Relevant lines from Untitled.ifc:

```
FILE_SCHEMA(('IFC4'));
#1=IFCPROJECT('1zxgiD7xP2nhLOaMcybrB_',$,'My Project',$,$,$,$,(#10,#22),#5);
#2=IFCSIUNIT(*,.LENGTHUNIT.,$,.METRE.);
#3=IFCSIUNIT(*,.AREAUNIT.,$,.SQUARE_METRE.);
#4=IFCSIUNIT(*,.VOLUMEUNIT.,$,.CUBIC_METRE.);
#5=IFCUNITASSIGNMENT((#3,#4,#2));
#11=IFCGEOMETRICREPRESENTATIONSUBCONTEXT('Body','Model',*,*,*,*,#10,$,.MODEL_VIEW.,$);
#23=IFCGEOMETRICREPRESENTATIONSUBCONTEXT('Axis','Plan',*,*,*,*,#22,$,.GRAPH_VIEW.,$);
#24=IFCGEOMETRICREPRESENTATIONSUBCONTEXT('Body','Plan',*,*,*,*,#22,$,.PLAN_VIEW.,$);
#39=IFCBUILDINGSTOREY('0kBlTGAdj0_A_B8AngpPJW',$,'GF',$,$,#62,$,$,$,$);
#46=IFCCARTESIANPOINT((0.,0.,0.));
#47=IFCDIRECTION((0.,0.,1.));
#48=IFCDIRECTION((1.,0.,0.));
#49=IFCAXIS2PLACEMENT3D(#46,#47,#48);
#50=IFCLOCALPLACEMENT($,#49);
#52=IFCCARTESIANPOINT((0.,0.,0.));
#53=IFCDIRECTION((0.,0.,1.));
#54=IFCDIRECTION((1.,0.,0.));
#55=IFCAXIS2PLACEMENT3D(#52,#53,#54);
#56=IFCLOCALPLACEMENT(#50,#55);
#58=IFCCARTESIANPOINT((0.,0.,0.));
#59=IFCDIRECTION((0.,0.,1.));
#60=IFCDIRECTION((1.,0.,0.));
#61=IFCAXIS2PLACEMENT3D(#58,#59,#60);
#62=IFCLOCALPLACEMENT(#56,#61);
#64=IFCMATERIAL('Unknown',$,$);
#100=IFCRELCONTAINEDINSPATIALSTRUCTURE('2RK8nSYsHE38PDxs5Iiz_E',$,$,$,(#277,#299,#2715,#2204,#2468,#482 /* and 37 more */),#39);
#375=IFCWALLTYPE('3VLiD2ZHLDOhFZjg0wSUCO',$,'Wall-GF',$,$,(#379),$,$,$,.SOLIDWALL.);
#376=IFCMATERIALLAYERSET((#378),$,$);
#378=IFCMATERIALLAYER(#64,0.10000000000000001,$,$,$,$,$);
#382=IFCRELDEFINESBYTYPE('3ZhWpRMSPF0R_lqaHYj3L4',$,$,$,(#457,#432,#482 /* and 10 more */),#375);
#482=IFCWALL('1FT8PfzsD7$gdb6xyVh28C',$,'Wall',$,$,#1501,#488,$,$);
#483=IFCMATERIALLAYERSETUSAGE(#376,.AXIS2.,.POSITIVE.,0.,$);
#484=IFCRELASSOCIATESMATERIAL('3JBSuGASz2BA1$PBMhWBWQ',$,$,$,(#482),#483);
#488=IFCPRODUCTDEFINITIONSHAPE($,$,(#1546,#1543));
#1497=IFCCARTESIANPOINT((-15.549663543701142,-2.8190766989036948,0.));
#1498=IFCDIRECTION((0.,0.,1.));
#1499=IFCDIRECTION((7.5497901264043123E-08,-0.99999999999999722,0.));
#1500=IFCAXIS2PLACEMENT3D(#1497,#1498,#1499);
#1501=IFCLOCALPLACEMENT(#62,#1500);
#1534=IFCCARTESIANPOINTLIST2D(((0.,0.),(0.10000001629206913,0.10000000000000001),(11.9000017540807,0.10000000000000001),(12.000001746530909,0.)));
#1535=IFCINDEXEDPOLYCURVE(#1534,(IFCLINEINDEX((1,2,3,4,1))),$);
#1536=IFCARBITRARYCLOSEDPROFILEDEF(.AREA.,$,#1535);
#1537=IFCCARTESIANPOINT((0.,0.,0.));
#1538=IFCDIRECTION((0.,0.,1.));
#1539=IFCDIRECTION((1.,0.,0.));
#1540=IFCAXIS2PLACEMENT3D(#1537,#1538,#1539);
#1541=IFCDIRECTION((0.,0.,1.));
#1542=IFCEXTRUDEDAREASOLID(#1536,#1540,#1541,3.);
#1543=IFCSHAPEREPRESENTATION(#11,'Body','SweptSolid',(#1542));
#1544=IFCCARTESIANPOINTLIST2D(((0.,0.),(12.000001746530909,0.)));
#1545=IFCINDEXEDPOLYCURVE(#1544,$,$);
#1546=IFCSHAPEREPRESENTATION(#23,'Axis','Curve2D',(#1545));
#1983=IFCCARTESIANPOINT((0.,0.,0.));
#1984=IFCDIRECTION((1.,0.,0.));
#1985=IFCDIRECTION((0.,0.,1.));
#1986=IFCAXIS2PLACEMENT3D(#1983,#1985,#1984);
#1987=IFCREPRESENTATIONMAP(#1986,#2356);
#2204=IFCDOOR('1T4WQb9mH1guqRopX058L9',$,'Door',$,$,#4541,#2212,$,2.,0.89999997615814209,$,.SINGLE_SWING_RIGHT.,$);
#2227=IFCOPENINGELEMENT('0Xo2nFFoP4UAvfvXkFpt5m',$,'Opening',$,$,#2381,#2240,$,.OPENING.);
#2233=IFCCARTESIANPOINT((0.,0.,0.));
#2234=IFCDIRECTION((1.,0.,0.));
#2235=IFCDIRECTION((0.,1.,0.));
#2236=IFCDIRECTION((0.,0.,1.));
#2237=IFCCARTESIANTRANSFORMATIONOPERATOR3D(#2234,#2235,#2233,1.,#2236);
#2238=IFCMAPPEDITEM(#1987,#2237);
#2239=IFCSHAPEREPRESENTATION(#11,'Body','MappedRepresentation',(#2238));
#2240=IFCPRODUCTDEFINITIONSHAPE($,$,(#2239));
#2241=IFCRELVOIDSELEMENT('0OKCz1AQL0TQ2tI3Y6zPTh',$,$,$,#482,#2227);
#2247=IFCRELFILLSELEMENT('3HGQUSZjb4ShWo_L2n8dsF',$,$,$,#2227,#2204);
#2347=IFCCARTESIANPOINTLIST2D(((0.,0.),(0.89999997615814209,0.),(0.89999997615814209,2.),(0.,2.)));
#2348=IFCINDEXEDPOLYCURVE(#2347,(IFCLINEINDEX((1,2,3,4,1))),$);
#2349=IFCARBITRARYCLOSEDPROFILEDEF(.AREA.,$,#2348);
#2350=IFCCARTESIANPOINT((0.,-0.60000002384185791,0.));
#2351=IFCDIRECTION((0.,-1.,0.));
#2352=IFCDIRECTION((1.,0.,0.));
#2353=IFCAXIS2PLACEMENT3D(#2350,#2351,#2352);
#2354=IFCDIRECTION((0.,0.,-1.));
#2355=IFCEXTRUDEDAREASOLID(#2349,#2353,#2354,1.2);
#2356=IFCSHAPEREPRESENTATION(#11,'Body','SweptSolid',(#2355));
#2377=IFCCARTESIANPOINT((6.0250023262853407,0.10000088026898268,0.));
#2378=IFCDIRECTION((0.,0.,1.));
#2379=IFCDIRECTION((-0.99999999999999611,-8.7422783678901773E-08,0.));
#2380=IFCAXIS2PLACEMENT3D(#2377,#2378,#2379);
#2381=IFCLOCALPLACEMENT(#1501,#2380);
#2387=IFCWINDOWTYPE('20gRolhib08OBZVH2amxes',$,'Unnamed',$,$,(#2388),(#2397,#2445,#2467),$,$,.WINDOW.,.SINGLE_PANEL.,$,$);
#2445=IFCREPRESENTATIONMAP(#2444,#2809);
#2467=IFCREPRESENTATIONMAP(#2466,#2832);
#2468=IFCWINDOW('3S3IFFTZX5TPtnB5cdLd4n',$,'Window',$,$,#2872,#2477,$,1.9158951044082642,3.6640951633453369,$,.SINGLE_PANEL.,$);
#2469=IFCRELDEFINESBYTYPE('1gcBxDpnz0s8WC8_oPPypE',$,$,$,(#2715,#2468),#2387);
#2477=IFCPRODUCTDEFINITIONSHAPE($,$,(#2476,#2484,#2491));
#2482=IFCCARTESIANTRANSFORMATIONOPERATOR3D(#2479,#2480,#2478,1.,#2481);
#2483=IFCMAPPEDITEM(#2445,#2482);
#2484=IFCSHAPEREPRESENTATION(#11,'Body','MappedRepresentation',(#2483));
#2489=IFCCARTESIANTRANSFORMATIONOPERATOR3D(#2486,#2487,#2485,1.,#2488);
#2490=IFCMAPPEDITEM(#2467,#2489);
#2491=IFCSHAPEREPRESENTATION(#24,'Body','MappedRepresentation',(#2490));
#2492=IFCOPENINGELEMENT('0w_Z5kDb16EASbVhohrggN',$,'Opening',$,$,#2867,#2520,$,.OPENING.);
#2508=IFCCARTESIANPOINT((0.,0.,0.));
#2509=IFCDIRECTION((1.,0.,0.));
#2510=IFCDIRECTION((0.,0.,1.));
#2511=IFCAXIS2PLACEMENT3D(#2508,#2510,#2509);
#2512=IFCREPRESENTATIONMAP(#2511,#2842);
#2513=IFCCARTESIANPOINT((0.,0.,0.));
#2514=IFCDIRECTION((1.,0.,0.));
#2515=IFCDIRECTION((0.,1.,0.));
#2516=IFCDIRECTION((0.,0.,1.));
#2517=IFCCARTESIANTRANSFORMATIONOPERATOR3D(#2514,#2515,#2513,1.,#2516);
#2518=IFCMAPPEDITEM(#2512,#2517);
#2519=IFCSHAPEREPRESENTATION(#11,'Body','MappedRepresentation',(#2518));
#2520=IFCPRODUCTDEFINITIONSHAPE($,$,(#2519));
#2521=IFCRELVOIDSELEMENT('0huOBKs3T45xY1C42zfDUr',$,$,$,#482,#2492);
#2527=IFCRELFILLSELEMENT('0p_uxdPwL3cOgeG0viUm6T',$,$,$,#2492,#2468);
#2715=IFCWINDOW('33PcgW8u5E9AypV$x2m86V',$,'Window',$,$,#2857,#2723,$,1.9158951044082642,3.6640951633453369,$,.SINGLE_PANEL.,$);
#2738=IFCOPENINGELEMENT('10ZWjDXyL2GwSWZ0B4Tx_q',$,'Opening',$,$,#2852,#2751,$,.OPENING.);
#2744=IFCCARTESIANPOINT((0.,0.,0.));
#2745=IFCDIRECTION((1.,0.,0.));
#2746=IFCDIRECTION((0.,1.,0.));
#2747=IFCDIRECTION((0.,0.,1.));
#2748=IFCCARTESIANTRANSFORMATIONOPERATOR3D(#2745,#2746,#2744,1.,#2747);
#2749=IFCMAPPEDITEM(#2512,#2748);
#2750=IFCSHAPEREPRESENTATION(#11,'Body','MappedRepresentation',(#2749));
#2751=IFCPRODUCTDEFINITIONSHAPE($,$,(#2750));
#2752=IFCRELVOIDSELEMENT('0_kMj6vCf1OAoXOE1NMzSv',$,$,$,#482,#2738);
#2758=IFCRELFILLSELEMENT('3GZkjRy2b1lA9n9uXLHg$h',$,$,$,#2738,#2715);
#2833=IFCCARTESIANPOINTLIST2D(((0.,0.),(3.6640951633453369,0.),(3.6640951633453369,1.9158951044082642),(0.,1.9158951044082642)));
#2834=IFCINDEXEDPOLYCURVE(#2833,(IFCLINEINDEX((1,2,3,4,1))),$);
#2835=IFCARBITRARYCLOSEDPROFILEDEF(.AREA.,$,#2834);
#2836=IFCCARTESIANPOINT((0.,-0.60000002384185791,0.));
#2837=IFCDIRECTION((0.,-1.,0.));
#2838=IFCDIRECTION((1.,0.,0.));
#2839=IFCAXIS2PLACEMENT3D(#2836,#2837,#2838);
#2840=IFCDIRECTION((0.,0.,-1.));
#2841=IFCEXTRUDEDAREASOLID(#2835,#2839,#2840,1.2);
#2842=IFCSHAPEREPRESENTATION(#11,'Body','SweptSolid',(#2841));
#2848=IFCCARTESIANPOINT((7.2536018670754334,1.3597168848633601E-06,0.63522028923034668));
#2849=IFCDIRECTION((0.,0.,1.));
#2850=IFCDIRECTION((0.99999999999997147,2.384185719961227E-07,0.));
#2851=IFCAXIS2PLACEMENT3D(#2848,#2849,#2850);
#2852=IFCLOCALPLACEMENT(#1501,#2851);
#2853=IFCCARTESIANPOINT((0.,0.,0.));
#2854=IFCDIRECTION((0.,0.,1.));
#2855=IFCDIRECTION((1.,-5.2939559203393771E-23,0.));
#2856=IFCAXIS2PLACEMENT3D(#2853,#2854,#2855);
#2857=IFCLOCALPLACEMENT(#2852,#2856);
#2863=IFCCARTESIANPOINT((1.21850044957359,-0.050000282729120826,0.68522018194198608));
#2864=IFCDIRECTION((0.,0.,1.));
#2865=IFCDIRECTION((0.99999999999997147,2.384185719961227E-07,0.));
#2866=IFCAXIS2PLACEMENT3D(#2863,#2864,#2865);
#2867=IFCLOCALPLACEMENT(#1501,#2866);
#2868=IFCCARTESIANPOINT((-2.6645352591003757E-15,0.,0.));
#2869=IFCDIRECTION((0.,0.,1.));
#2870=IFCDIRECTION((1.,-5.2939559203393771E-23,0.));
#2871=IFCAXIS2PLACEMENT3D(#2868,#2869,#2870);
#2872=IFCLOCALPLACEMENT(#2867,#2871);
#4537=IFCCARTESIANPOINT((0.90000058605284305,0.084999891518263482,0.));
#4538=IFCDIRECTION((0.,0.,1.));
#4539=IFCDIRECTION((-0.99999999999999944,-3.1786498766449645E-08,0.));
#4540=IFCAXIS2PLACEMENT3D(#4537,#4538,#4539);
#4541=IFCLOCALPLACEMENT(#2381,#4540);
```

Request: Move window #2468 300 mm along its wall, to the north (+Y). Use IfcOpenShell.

```python
import ifcopenshell
import ifcopenshell.api.geometry
import ifcopenshell.util.placement

model = ifcopenshell.open("Untitled.ifc")

window = model.by_guid("3S3IFFTZX5TPtnB5cdLd4n")
opening = window.FillsVoids[0].RelatingOpeningElement
wall = opening.VoidsElements[0].RelatingBuildingElement

wall_matrix = ifcopenshell.util.placement.get_local_placement(wall.ObjectPlacement)
shift = wall_matrix[:3, 0] * -0.3
before = ifcopenshell.util.placement.get_local_placement(window.ObjectPlacement)[:3, 3].copy()

# The window is placed relative to its opening, so it follows when the opening moves.
matrix = ifcopenshell.util.placement.get_local_placement(opening.ObjectPlacement)
matrix[:3, 3] += shift
ifcopenshell.api.geometry.edit_object_placement(
    model, product=opening, matrix=matrix, is_si=False, should_transform_children=True
)

after = ifcopenshell.util.placement.get_local_placement(window.ObjectPlacement)[:3, 3]
print("window moved by", (after - before).round(3) + 0.0)

model.write("Untitled_rev.ifc")
```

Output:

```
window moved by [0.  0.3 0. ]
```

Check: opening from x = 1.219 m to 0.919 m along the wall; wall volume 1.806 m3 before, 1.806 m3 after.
